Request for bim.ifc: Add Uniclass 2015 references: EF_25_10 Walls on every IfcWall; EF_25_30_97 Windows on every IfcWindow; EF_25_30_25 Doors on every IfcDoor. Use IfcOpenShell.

First a look at what the model holds.

```python
import ifcopenshell

model = ifcopenshell.open("bim.ifc")
print(model.schema)
print("classifications:", [c.Name for c in model.by_type("IfcClassification")])
for ifc_class in ("IfcDoor", "IfcRoof", "IfcStair", "IfcWall", "IfcWindow"):
    print(ifc_class, len(model.by_type(ifc_class)))
```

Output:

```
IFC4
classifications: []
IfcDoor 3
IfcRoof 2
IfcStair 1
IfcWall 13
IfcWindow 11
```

```python
import ifcopenshell
import ifcopenshell.api.classification

model = ifcopenshell.open("bim.ifc")

system = ifcopenshell.api.classification.add_classification(model, classification="Uniclass 2015")

codes = {
    "IfcWall": ("EF_25_10", "Walls"),
    "IfcWindow": ("EF_25_30_97", "Windows"),
    "IfcDoor": ("EF_25_30_25", "Doors"),
}
for ifc_class, (code, name) in codes.items():
    products = model.by_type(ifc_class)
    ifcopenshell.api.classification.add_reference(
        model, products=products, classification=system, identification=code, name=name
    )
    print(code, len(products))

model.write("bim_rev.ifc")
```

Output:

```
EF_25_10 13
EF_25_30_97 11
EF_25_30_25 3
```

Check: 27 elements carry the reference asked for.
